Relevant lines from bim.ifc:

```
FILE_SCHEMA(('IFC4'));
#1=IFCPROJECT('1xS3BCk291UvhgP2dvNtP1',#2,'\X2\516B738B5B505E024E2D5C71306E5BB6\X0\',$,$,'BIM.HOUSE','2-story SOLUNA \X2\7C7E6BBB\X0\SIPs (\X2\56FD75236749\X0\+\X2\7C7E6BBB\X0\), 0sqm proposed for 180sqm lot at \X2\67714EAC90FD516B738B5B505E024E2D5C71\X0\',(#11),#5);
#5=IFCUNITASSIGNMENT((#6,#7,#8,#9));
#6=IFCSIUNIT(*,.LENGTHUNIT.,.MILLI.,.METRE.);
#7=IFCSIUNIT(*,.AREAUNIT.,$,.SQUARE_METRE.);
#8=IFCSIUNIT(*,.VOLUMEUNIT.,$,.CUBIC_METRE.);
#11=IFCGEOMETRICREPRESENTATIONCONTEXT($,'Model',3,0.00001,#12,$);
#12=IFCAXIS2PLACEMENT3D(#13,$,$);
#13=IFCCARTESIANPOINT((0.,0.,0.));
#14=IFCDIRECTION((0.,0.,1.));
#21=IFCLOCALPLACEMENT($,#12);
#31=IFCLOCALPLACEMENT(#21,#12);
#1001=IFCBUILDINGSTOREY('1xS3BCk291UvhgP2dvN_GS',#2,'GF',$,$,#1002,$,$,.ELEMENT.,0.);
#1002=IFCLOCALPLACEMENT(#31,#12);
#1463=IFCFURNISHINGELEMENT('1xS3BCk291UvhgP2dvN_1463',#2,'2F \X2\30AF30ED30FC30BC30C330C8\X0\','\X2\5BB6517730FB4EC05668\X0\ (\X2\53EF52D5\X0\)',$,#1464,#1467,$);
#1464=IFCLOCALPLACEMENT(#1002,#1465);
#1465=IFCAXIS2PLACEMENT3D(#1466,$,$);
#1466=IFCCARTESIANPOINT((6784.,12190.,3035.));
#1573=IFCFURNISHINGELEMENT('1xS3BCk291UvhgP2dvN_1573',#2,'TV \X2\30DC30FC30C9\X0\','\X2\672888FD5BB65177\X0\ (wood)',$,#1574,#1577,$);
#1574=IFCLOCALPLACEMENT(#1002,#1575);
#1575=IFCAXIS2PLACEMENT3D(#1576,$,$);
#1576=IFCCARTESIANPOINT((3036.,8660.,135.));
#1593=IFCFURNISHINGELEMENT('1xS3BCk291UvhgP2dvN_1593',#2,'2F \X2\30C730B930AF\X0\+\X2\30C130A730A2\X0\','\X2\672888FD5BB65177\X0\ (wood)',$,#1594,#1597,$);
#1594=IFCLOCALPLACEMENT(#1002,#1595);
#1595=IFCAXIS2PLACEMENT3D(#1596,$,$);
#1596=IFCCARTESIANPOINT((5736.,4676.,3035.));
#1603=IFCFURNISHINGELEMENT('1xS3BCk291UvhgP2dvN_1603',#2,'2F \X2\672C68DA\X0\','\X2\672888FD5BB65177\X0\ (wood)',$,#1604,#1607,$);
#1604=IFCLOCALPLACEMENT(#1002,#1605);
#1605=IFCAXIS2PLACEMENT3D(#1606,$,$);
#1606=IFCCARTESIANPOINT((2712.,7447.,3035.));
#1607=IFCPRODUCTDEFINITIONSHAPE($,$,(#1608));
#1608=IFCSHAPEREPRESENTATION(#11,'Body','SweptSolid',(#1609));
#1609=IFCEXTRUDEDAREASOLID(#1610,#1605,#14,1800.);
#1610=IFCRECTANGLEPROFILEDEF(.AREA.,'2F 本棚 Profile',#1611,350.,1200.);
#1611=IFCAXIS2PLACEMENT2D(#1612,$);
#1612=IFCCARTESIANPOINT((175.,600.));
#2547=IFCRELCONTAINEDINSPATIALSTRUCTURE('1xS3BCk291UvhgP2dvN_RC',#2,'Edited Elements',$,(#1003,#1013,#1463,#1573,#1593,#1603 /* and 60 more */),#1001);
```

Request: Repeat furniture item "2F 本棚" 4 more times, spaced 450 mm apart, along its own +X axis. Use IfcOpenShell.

```python
import ifcopenshell
import ifcopenshell.api.geometry
import ifcopenshell.api.root
import ifcopenshell.util.element
import ifcopenshell.util.placement
import ifcopenshell.util.unit

model = ifcopenshell.open("bim.ifc")
unit_scale = ifcopenshell.util.unit.calculate_unit_scale(model)


def reuse_history(source, copy):
    """copy_class also copies each property set's owner history, people and application; keep the originals."""
    for rel in copy.IsDefinedBy:
        if rel.is_a("IfcRelDefinesByProperties") and (history := rel.RelatingPropertyDefinition.OwnerHistory):
            rel.RelatingPropertyDefinition.OwnerHistory = source.OwnerHistory
            ifcopenshell.util.element.remove_deep2(model, history)


source = model.by_guid("1xS3BCk291UvhgP2dvN_1603")
base = ifcopenshell.util.placement.get_local_placement(source.ObjectPlacement)
step = base[:3, 0] * 0.45 / unit_scale

for i in range(1, 5):
    copy = ifcopenshell.api.root.copy_class(model, product=source)
    copy.Representation = ifcopenshell.util.element.copy_deep(
        model, source.Representation, exclude=["IfcGeometricRepresentationContext", "IfcRepresentationMap"]
    )
    reuse_history(source, copy)
    matrix = base.copy()
    matrix[:3, 3] += i * step
    print("added at", matrix[:3, 3].round(3) + 0.0)
    ifcopenshell.api.geometry.edit_object_placement(model, product=copy, matrix=matrix, is_si=False)

model.write("bim_v2.ifc")
```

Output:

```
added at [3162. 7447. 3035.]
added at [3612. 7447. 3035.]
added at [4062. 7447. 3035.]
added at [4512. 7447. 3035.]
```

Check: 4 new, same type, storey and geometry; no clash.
